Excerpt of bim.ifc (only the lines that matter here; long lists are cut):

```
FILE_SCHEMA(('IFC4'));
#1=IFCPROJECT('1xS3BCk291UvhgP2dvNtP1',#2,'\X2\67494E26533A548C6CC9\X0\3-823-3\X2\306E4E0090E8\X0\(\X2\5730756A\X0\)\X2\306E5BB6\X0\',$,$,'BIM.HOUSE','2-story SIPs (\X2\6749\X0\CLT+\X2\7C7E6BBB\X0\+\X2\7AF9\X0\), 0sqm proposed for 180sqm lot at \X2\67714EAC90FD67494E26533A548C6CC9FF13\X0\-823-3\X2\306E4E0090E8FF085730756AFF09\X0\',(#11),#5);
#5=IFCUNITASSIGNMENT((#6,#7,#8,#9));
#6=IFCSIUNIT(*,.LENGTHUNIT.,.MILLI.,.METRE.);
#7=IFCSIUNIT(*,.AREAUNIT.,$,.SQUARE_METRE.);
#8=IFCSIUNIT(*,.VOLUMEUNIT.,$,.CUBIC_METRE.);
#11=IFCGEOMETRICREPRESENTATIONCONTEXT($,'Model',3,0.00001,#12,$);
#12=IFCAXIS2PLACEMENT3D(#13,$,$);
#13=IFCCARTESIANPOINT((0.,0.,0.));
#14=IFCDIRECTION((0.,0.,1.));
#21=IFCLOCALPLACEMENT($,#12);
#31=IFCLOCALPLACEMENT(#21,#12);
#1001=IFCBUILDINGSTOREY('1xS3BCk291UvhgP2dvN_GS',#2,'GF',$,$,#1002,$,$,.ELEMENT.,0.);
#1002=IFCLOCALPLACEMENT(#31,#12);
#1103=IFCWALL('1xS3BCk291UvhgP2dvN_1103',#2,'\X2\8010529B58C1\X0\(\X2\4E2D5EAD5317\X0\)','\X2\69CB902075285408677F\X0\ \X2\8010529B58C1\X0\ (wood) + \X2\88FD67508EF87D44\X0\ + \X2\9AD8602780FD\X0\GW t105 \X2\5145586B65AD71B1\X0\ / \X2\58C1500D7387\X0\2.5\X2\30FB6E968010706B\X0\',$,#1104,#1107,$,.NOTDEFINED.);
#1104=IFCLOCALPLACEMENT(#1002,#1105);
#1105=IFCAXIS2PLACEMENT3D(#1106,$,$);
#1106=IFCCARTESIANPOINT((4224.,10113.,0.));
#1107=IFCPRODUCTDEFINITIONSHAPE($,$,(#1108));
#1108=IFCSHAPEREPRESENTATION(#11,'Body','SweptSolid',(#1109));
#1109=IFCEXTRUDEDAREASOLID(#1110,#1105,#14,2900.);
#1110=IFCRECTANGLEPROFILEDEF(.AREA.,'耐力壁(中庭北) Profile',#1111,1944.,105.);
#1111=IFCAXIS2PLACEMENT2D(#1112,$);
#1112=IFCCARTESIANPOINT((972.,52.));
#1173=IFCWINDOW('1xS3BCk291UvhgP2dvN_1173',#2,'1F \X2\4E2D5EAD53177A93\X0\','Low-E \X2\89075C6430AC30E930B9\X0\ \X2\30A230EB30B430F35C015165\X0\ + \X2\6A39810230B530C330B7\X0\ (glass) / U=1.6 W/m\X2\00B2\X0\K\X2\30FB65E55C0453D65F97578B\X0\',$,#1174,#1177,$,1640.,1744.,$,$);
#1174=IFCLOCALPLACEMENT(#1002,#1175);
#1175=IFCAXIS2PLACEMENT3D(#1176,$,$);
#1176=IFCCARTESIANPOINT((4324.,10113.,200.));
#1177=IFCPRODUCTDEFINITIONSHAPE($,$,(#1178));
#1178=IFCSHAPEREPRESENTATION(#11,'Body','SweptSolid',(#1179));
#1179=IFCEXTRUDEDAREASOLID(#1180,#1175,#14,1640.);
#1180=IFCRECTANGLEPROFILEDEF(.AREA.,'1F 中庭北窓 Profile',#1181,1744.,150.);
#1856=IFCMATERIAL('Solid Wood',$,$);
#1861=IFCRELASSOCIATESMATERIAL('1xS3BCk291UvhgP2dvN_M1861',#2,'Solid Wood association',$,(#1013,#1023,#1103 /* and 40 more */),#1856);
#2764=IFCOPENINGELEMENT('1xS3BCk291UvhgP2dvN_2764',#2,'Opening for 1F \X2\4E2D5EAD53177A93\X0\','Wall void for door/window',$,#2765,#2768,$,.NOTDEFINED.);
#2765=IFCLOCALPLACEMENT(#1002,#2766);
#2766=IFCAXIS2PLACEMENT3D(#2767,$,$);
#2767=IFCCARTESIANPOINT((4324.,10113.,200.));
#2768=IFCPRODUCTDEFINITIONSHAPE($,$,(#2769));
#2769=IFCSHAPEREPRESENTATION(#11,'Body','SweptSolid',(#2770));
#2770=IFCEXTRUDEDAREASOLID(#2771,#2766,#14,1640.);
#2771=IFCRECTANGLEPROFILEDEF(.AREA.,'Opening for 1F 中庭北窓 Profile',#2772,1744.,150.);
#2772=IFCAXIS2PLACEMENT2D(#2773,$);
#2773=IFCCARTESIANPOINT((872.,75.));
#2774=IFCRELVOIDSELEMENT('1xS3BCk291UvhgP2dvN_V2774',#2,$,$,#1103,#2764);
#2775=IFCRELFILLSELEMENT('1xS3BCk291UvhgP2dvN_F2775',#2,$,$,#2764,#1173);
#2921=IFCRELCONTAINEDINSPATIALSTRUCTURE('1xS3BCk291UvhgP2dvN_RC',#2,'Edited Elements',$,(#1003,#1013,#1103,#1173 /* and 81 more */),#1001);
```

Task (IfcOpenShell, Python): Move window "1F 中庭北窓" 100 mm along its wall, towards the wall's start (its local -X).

```python
import ifcopenshell
import ifcopenshell.api.geometry
import ifcopenshell.util.placement
import ifcopenshell.util.unit

model = ifcopenshell.open("bim.ifc")
unit_scale = ifcopenshell.util.unit.calculate_unit_scale(model)

window = model.by_guid("1xS3BCk291UvhgP2dvN_1173")
opening = window.FillsVoids[0].RelatingOpeningElement
wall = opening.VoidsElements[0].RelatingBuildingElement

wall_matrix = ifcopenshell.util.placement.get_local_placement(wall.ObjectPlacement)
shift = wall_matrix[:3, 0] * -0.1 / unit_scale
before = ifcopenshell.util.placement.get_local_placement(window.ObjectPlacement)[:3, 3].copy()

# The window is not placed relative to its opening, so move both.
for product in (opening, window):
    matrix = ifcopenshell.util.placement.get_local_placement(product.ObjectPlacement)
    matrix[:3, 3] += shift
    ifcopenshell.api.geometry.edit_object_placement(model, product=product, matrix=matrix, is_si=False)

after = ifcopenshell.util.placement.get_local_placement(window.ObjectPlacement)[:3, 3]
print("window moved by", (after - before).round(3) + 0.0)

model.write("bim_updated.ifc")
```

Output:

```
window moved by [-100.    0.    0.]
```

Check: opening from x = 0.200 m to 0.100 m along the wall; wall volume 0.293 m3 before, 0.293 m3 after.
